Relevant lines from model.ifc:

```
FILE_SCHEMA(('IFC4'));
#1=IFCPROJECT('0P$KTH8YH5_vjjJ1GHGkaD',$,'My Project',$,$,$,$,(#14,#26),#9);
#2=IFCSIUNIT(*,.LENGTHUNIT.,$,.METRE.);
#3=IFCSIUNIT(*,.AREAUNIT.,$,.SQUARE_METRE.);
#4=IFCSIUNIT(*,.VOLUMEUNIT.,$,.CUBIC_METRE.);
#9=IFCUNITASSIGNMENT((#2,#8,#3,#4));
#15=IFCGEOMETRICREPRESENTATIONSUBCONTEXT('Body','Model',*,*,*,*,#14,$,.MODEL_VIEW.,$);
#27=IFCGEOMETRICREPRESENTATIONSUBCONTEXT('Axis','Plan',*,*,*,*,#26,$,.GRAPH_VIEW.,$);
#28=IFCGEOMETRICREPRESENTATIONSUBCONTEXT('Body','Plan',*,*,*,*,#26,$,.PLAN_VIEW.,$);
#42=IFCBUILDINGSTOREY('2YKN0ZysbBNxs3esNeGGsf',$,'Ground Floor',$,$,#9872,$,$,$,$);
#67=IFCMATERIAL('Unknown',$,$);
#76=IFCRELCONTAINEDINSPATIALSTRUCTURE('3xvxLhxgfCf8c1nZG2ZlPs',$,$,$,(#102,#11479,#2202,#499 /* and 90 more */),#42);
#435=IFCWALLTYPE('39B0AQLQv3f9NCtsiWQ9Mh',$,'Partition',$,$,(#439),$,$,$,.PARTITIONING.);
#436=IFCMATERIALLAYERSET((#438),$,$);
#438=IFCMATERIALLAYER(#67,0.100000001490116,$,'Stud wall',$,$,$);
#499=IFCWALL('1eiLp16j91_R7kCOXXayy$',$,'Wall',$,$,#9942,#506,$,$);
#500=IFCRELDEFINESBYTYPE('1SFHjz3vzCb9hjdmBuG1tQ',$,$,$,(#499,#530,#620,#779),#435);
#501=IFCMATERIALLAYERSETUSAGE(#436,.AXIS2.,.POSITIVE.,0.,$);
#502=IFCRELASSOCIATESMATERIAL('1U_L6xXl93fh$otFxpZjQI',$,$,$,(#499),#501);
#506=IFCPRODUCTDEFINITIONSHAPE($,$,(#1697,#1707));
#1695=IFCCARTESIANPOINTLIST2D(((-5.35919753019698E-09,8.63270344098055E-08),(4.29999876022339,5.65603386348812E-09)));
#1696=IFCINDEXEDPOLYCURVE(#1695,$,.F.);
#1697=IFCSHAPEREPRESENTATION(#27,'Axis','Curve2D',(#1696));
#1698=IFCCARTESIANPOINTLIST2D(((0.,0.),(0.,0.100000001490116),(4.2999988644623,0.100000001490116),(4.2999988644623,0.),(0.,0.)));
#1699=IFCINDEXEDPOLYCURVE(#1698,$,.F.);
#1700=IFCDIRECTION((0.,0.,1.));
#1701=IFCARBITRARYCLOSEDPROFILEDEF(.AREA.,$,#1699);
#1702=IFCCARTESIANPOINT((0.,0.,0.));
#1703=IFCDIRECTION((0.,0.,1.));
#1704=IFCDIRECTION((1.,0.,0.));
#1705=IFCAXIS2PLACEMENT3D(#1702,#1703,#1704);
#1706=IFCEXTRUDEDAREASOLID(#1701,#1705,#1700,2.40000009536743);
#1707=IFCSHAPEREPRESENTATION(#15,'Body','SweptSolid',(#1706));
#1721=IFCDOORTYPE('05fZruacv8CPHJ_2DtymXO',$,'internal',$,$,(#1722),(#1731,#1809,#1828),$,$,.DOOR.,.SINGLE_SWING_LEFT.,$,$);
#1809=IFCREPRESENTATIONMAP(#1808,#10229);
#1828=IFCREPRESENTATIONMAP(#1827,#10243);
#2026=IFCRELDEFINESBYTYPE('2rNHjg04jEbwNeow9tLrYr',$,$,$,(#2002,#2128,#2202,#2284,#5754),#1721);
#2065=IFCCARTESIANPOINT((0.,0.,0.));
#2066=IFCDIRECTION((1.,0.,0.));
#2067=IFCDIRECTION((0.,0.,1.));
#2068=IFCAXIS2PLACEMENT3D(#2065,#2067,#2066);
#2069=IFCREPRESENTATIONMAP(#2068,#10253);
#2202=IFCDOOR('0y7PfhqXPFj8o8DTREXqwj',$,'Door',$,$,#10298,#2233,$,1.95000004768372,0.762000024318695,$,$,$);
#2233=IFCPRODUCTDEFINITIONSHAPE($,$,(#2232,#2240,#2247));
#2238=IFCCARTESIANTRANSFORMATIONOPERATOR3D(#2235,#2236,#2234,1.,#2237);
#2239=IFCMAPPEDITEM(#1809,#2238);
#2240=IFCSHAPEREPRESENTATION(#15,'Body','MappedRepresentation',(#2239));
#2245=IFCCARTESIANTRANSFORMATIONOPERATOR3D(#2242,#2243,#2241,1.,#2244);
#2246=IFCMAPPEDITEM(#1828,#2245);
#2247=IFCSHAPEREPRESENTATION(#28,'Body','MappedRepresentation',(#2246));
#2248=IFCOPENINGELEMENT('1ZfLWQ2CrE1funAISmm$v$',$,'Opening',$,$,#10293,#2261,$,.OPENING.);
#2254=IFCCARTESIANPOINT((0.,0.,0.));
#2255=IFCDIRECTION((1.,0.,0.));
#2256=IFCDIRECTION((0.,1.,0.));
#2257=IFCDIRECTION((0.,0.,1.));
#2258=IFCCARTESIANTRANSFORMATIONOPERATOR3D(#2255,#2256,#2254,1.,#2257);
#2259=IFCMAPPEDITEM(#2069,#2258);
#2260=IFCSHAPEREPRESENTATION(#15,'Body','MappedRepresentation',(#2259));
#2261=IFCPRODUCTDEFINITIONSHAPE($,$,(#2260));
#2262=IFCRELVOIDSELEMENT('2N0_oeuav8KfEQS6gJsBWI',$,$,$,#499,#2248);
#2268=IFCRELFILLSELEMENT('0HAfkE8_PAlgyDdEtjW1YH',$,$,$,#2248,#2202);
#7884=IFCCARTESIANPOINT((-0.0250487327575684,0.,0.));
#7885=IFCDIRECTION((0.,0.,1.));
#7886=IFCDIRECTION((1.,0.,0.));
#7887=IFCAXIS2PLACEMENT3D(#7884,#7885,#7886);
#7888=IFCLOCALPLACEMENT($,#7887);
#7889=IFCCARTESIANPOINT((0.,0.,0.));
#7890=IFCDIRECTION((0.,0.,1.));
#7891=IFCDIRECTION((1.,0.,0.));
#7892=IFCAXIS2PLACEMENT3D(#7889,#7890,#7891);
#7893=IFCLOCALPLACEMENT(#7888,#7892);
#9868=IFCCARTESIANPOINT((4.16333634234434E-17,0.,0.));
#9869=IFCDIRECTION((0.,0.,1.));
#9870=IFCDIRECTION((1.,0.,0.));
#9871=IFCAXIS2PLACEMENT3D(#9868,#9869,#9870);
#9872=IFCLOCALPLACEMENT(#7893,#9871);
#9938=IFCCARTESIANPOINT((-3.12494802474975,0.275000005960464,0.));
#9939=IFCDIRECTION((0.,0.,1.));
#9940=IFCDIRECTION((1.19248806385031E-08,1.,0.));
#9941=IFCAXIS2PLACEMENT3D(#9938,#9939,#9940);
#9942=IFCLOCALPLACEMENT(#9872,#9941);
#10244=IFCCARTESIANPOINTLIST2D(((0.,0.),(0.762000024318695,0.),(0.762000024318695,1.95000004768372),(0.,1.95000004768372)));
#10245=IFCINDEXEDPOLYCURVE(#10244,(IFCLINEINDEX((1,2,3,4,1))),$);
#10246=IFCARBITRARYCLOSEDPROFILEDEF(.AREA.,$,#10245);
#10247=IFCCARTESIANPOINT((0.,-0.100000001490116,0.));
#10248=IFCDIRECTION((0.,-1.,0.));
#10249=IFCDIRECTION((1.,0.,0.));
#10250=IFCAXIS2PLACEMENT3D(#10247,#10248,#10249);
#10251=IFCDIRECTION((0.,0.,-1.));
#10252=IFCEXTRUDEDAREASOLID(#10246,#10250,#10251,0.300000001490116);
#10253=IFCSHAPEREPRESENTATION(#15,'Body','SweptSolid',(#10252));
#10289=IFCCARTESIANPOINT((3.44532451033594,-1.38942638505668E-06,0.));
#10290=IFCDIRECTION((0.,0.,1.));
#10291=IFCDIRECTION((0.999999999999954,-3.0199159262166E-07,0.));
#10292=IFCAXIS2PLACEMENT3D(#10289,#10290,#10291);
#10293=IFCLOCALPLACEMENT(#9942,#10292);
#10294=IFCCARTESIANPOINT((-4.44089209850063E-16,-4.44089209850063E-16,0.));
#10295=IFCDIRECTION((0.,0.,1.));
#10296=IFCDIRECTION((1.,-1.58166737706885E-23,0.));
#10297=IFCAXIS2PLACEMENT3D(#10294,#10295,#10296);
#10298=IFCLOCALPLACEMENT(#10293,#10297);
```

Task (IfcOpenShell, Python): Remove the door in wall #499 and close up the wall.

```python
import ifcopenshell
import ifcopenshell.api.feature
import ifcopenshell.api.root
import ifcopenshell.geom
import ifcopenshell.util.shape

model = ifcopenshell.open("model.ifc")
settings = ifcopenshell.geom.settings()


def volume(element):
    """Net volume in cubic metres, openings subtracted."""
    shape = ifcopenshell.geom.create_shape(settings, element)
    return ifcopenshell.util.shape.get_volume(shape.geometry)


door = model.by_guid("0y7PfhqXPFj8o8DTREXqwj")
opening = door.FillsVoids[0].RelatingOpeningElement
wall = opening.VoidsElements[0].RelatingBuildingElement
before = volume(wall)

ifcopenshell.api.root.remove_product(model, product=door)
ifcopenshell.api.feature.remove_feature(model, feature=opening)

after = volume(wall)

print(f"wall volume {before:.3f} -> {after:.3f} m3")

model.write("model_updated.ifc")
```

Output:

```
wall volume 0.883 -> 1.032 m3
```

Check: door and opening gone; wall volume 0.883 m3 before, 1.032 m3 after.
